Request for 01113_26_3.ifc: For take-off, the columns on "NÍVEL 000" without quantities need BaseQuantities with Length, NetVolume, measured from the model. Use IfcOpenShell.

First a look at what the model holds.

```python
import ifcopenshell
import ifcopenshell.util.element
import ifcopenshell.util.unit

model = ifcopenshell.open("01113_26_3.ifc")
print(model.schema)
for unit_type in ("LENGTHUNIT", "AREAUNIT", "VOLUMEUNIT"):
    print(unit_type, ifcopenshell.util.unit.calculate_unit_scale(model, unit_type))
storey = next(s for s in model.by_type("IfcBuildingStorey") if s.Name == "NÍVEL 000")
columns = [e for e in ifcopenshell.util.element.get_decomposition(storey) if e.is_a("IfcColumn")]
for e in sorted(columns, key=lambda e: e.id()):
    print(e.id(), e.is_a(), e.Name, list(ifcopenshell.util.element.get_psets(e, qtos_only=True)), sep=" | ")
```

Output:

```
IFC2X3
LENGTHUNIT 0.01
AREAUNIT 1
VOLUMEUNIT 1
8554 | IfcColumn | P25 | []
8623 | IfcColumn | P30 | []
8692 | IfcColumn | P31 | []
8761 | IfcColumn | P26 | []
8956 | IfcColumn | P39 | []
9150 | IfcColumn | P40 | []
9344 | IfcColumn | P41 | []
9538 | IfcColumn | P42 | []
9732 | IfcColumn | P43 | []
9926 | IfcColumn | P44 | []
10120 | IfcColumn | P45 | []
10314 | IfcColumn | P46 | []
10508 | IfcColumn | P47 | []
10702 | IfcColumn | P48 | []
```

```python
import ifcopenshell
import ifcopenshell.api.pset
import ifcopenshell.geom
import ifcopenshell.util.element
import ifcopenshell.util.shape
import ifcopenshell.util.unit

model = ifcopenshell.open("01113_26_3.ifc")
unit_scale = ifcopenshell.util.unit.calculate_unit_scale(model)
volume_scale = ifcopenshell.util.unit.calculate_unit_scale(model, "VOLUMEUNIT")
settings = ifcopenshell.geom.settings()

storey = next(s for s in model.by_type("IfcBuildingStorey") if s.Name == "NÍVEL 000")
columns = [e for e in ifcopenshell.util.element.get_decomposition(storey) if e.is_a("IfcColumn")]

for e in sorted(columns, key=lambda e: e.id()):
    if ifcopenshell.util.element.get_psets(e, qtos_only=True, should_inherit=False):
        continue
    # Geometry comes back in metres, in the element's own axes.
    shape = ifcopenshell.geom.create_shape(settings, e)
    values = {
        "Length": ifcopenshell.util.shape.get_z(shape.geometry) / unit_scale,
        "NetVolume": ifcopenshell.util.shape.get_volume(shape.geometry) / volume_scale,
    }
    qto = ifcopenshell.api.pset.add_qto(model, product=e, name="BaseQuantities")
    ifcopenshell.api.pset.edit_qto(model, qto=qto, properties=values)
    print(e.id(), {k: round(v, 3) for k, v in values.items()})

model.write("01113_26_3_edited.ifc")
```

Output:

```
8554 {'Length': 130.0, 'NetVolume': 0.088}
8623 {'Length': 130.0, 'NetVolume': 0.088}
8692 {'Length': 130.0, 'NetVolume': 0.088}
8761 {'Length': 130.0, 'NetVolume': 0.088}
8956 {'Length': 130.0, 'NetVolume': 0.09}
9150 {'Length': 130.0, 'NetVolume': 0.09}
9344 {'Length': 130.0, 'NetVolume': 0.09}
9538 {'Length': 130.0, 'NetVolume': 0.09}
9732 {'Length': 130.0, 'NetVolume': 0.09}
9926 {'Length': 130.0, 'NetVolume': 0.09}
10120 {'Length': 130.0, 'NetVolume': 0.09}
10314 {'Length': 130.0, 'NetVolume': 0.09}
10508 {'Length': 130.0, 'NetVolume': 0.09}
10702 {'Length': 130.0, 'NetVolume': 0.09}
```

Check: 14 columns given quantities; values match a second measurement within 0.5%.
